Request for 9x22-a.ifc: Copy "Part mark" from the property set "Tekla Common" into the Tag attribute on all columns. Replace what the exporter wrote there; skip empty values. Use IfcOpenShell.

First a look at what the model holds.

```python
import ifcopenshell
import ifcopenshell.util.element

model = ifcopenshell.open("9x22-a.ifc")
print(model.schema)
columns = model.by_type("IfcColumn")
print(len(columns), "columns")
for e in columns[:8]:
    source = ifcopenshell.util.element.get_pset(e, "Tekla Common", "Part mark")
    target = e.Tag
    print(e.id(), repr(source), repr(target), sep=" | ")
```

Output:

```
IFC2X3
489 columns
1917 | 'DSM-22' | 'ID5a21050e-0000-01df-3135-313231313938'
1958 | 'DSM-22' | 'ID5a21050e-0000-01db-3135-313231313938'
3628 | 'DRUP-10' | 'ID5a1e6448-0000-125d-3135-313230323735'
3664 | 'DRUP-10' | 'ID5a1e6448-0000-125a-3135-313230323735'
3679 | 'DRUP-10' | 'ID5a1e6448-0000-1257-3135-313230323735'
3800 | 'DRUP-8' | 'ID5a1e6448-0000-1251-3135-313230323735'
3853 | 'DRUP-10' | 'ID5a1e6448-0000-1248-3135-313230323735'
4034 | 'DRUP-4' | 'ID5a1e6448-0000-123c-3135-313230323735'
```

```python
import ifcopenshell
import ifcopenshell.util.element

model = ifcopenshell.open("9x22-a.ifc")

count = 0
for e in model.by_type("IfcColumn"):
    value = ifcopenshell.util.element.get_pset(e, "Tekla Common", "Part mark")
    current = e.Tag
    if not value or not value.strip() or current == value:
        continue
    e.Tag = value
    count += 1

print(count, "columns updated")

model.write("9x22-a_v2.ifc")
```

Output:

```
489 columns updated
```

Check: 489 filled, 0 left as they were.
